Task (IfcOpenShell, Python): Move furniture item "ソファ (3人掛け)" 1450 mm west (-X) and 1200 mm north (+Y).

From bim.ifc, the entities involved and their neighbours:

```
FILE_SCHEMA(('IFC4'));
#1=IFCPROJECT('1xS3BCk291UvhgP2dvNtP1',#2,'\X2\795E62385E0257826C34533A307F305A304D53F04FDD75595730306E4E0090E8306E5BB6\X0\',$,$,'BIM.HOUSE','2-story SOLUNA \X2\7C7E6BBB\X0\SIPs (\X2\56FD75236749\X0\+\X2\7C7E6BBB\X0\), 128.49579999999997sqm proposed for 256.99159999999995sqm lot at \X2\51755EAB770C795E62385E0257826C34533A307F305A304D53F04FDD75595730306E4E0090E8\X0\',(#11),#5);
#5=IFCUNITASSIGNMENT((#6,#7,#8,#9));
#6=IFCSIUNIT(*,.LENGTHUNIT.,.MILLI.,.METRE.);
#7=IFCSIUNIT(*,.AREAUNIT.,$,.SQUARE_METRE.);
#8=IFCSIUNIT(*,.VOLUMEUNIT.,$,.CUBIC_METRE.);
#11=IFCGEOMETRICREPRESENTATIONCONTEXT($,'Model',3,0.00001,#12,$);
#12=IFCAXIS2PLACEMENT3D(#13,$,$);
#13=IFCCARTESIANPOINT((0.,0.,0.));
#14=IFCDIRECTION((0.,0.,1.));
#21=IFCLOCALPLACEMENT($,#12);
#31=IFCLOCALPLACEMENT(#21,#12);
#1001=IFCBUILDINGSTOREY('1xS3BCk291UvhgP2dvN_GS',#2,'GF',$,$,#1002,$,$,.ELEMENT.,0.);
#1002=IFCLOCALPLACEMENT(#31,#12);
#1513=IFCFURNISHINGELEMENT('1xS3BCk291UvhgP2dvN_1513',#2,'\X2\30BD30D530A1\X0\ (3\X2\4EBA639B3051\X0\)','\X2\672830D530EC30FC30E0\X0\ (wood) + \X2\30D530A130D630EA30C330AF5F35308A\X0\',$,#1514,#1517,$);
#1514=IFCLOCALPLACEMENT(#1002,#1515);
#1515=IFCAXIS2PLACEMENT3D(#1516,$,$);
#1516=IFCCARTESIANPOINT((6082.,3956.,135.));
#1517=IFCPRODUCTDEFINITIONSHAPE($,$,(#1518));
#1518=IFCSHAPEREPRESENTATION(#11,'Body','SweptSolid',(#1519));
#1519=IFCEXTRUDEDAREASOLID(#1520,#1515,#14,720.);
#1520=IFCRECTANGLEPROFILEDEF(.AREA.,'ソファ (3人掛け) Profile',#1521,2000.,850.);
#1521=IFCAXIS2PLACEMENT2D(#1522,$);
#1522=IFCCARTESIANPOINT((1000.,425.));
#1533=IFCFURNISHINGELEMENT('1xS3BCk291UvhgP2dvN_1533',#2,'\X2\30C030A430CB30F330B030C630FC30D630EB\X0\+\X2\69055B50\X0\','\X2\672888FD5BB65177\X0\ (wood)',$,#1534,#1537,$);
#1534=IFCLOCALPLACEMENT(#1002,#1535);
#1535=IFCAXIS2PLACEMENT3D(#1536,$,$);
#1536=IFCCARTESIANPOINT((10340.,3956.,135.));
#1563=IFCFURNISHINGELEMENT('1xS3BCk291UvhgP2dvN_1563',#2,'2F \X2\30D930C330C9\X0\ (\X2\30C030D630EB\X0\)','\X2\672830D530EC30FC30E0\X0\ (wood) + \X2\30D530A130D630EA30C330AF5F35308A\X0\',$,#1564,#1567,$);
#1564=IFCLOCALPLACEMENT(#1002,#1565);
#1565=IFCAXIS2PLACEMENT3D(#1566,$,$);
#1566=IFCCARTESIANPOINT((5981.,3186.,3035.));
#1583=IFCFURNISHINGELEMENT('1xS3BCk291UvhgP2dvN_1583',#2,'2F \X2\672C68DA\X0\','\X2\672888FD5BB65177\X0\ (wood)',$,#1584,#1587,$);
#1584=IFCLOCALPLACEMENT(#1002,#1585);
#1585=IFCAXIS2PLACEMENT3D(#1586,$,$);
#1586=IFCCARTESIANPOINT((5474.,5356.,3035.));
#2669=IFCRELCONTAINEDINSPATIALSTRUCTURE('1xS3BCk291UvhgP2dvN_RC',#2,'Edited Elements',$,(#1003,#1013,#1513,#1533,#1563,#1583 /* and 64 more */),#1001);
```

```python
import ifcopenshell
import ifcopenshell.api.geometry
import ifcopenshell.util.placement
import ifcopenshell.util.unit

model = ifcopenshell.open("bim.ifc")
unit_scale = ifcopenshell.util.unit.calculate_unit_scale(model)

item = model.by_guid("1xS3BCk291UvhgP2dvN_1513")
matrix = ifcopenshell.util.placement.get_local_placement(item.ObjectPlacement)
matrix[0, 3] -= 1.45 / unit_scale
matrix[1, 3] += 1.2 / unit_scale
ifcopenshell.api.geometry.edit_object_placement(model, product=item, matrix=matrix, is_si=False)

print(ifcopenshell.util.placement.get_local_placement(item.ObjectPlacement).round(3) + 0.0)

model.write("bim_v2.ifc")
```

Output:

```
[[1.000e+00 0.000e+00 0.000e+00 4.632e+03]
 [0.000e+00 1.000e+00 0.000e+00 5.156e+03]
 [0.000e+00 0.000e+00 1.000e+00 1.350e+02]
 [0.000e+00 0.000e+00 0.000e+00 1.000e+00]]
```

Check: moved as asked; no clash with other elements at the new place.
